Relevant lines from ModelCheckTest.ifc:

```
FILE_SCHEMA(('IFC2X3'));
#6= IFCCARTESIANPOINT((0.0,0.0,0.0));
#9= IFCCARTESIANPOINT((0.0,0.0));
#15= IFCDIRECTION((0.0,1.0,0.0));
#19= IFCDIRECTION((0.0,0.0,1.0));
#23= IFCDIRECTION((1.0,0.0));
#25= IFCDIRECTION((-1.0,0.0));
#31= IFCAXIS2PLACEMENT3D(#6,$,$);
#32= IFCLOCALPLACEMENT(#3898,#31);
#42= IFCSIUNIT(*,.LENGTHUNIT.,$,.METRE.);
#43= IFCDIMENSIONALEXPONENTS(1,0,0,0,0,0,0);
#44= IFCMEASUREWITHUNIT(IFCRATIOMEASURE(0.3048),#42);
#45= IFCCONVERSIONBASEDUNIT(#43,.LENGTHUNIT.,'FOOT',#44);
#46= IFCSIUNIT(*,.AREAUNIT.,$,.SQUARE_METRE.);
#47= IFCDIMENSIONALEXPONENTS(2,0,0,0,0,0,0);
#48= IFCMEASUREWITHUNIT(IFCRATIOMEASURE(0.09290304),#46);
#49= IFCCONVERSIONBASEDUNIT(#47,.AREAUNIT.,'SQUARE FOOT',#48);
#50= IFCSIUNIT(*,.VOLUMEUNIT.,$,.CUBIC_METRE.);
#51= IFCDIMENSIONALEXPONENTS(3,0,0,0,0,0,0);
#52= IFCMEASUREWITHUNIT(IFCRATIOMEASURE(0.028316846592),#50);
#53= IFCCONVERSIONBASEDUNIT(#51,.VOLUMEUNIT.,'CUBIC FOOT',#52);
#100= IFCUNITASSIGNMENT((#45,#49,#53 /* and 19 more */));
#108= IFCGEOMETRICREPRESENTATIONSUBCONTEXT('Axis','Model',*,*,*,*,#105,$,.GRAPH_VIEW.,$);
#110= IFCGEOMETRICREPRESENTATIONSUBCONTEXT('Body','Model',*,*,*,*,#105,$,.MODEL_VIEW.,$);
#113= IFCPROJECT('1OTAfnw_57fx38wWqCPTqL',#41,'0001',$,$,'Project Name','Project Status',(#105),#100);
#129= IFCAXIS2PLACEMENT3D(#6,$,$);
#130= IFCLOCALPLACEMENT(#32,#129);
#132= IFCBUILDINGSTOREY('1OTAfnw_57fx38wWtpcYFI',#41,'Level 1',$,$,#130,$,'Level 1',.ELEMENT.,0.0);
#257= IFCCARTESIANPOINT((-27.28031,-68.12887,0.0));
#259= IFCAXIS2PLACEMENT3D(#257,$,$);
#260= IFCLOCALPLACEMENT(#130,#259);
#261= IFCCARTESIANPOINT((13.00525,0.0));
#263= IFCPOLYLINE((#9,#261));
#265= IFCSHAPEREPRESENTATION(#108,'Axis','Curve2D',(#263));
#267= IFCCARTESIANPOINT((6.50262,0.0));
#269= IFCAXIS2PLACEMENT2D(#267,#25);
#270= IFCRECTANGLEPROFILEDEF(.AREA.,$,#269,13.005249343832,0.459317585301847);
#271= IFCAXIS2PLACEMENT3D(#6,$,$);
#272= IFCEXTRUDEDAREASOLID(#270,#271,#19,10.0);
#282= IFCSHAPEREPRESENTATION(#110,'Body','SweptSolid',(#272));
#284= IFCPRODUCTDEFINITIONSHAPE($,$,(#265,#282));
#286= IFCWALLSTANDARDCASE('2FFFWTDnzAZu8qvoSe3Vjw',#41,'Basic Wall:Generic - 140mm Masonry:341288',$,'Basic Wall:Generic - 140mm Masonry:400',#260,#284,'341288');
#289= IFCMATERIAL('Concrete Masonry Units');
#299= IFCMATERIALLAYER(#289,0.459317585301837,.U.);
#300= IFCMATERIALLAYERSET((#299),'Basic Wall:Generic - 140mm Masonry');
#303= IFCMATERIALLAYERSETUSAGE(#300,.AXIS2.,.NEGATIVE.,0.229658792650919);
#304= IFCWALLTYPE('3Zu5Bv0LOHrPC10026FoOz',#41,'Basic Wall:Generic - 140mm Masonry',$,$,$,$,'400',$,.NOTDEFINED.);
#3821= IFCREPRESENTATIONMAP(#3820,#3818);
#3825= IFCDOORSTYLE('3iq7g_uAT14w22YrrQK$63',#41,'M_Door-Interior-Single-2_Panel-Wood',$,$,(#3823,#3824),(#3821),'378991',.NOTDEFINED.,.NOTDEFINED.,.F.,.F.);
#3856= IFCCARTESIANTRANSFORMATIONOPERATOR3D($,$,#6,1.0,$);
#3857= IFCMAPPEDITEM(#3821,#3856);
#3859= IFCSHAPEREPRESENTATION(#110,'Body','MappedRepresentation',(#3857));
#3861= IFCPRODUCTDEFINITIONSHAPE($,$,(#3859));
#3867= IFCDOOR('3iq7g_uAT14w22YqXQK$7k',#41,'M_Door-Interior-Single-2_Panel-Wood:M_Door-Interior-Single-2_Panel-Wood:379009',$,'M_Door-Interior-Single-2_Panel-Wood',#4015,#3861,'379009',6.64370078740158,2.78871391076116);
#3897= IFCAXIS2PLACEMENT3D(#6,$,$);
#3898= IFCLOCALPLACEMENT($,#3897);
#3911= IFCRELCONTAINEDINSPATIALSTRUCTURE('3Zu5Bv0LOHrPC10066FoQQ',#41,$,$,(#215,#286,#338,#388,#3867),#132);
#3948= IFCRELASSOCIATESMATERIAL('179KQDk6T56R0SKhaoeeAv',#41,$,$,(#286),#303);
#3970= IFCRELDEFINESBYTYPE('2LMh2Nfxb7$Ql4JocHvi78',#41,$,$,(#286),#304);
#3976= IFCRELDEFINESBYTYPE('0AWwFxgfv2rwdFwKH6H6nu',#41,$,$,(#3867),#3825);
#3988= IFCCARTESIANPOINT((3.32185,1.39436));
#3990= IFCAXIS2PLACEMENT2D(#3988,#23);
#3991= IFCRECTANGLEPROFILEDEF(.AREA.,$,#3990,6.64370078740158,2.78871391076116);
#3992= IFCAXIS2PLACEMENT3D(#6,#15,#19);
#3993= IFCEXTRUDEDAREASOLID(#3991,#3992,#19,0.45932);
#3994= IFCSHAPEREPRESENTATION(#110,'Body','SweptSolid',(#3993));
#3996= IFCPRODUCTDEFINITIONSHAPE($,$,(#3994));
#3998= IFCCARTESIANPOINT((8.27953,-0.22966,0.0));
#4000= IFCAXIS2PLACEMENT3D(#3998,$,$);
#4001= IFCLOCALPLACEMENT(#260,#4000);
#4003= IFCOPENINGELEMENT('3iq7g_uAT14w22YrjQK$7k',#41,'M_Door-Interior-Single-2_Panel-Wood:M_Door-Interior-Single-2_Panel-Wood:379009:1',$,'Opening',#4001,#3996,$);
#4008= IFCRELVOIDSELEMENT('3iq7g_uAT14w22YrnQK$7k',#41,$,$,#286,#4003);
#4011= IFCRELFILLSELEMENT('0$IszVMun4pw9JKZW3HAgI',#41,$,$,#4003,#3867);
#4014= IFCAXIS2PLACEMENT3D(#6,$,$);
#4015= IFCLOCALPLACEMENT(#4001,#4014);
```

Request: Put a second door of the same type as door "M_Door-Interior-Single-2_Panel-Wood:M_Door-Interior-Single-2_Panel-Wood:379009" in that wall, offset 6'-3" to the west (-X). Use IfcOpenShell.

```python
import ifcopenshell
import ifcopenshell.api.feature
import ifcopenshell.api.geometry
import ifcopenshell.api.root
import ifcopenshell.geom
import ifcopenshell.util.element
import ifcopenshell.util.placement
import ifcopenshell.util.shape
import ifcopenshell.util.unit

model = ifcopenshell.open("ModelCheckTest.ifc")
unit_scale = ifcopenshell.util.unit.calculate_unit_scale(model)
settings = ifcopenshell.geom.settings()


def volume(element):
    """Net volume in cubic metres, openings subtracted."""
    shape = ifcopenshell.geom.create_shape(settings, element)
    return ifcopenshell.util.shape.get_volume(shape.geometry)


def reuse_history(source, copy):
    """copy_class also copies each property set's owner history, people and application; keep the originals."""
    for rel in copy.IsDefinedBy:
        if rel.is_a("IfcRelDefinesByProperties") and (history := rel.RelatingPropertyDefinition.OwnerHistory):
            rel.RelatingPropertyDefinition.OwnerHistory = source.OwnerHistory
            ifcopenshell.util.element.remove_deep2(model, history)


door = model.by_id(3867)
opening = door.FillsVoids[0].RelatingOpeningElement
wall = opening.VoidsElements[0].RelatingBuildingElement
before = volume(wall)
shift = ifcopenshell.util.placement.get_local_placement(wall.ObjectPlacement)[:3, 0] * -75 * 0.0254 / unit_scale

# copy_class copies the void relationship, type, container and properties, but no geometry.
new_opening = ifcopenshell.api.root.copy_class(model, product=opening)
new_opening.Representation = ifcopenshell.util.element.copy_deep(
    model, opening.Representation, exclude=["IfcGeometricRepresentationContext", "IfcRepresentationMap"]
)
new_opening.Name = "M_Door-Interior-Single-2_Panel-Wood:M_Door-Interior-Single-2_Panel-Wood"
new_door = ifcopenshell.api.root.copy_class(model, product=door)
new_door.Representation = ifcopenshell.util.element.copy_deep(
    model, door.Representation, exclude=["IfcGeometricRepresentationContext", "IfcRepresentationMap"]
)
new_door.Name = "M_Door-Interior-Single-2_Panel-Wood:M_Door-Interior-Single-2_Panel-Wood"
new_door.Tag = None
reuse_history(door, new_door)
fills = ifcopenshell.api.feature.add_filling(model, opening=new_opening, element=new_door)
fills.OwnerHistory = new_door.OwnerHistory  # required in IFC2X3

for old, new in ((opening, new_opening), (door, new_door)):
    matrix = ifcopenshell.util.placement.get_local_placement(old.ObjectPlacement)
    matrix[:3, 3] += shift
    ifcopenshell.api.geometry.edit_object_placement(model, product=new, matrix=matrix, is_si=False)

after = volume(wall)

print(f"wall volume {before:.3f} -> {after:.3f} m3")

model.write("ModelCheckTest_rev.ifc")
```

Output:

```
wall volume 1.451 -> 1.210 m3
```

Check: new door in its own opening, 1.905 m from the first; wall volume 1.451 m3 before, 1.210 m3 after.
